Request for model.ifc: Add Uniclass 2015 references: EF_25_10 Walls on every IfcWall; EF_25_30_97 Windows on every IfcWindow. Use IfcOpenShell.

First a look at what the model holds.

```python
import ifcopenshell

model = ifcopenshell.open("model.ifc")
print(model.schema)
print("classifications:", [c.Name for c in model.by_type("IfcClassification")])
for ifc_class in ("IfcDoor", "IfcRoof", "IfcStair", "IfcWall", "IfcWindow"):
    print(ifc_class, len(model.by_type(ifc_class)))
```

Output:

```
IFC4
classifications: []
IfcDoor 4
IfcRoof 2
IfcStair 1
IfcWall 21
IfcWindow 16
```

```python
import ifcopenshell
import ifcopenshell.api.classification

model = ifcopenshell.open("model.ifc")

system = ifcopenshell.api.classification.add_classification(model, classification="Uniclass 2015")

codes = {
    "IfcWall": ("EF_25_10", "Walls"),
    "IfcWindow": ("EF_25_30_97", "Windows"),
}
for ifc_class, (code, name) in codes.items():
    products = model.by_type(ifc_class)
    ifcopenshell.api.classification.add_reference(
        model, products=products, classification=system, identification=code, name=name
    )
    print(code, len(products))

model.write("model_updated.ifc")
```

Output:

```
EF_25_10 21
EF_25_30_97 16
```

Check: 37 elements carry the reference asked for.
